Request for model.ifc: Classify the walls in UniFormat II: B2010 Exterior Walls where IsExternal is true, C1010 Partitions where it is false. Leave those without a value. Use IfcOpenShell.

First a look at what the model holds.

```python
import ifcopenshell
import ifcopenshell.util.element

model = ifcopenshell.open("model.ifc")
print(model.schema)
print("classifications:", [c.Name for c in model.by_type("IfcClassification")])
values = [ifcopenshell.util.element.get_pset(e, "Pset_WallCommon", "IsExternal") for e in model.by_type("IfcWall")]
for value in (True, False, None):
    print("IsExternal", value, values.count(value))
```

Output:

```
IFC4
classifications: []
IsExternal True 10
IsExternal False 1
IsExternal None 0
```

```python
import ifcopenshell
import ifcopenshell.api.classification
import ifcopenshell.util.element

model = ifcopenshell.open("model.ifc")

system = ifcopenshell.api.classification.add_classification(model, classification="UniFormat II")

walls = model.by_type("IfcWall")
external = {e: ifcopenshell.util.element.get_pset(e, "Pset_WallCommon", "IsExternal") for e in walls}
for flag, code, name in ((True, "B2010", "Exterior Walls"), (False, "C1010", "Partitions")):
    products = [e for e in walls if external[e] is flag]
    ifcopenshell.api.classification.add_reference(
        model, products=products, classification=system, identification=code, name=name
    )
    print(code, len(products))

model.write("model_v2.ifc")
```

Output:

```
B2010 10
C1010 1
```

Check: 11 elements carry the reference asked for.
